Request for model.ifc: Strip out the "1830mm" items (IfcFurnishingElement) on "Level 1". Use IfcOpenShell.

First a look at what the model holds.

```python
import ifcopenshell
import ifcopenshell.util.element

model = ifcopenshell.open("model.ifc")
print(model.schema)
storey = next(s for s in model.by_type("IfcBuildingStorey") if s.Name == "Level 1")
furniture = [e for e in ifcopenshell.util.element.get_decomposition(storey) if e.is_a("IfcFurnishingElement")]
seen = {}
for e in furniture:
    element_type = ifcopenshell.util.element.get_type(e)
    name = element_type.Name if element_type not in (None, e) else None
    seen[name] = seen.get(name, 0) + 1
for name, count in sorted(seen.items(), key=str):
    print(count, "x", name)
```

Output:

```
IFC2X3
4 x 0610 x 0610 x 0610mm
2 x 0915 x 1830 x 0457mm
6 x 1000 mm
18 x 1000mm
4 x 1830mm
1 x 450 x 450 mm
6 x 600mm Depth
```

```python
import ifcopenshell
import ifcopenshell.api.root
import ifcopenshell.util.element

model = ifcopenshell.open("model.ifc")

storey = next(s for s in model.by_type("IfcBuildingStorey") if s.Name == "Level 1")
furniture = [e for e in ifcopenshell.util.element.get_decomposition(storey) if e.is_a("IfcFurnishingElement")]
targets = [e for e in furniture if (t := ifcopenshell.util.element.get_type(e)) not in (None, e) and t.Name == "1830mm"]

for e in targets:
    ifcopenshell.api.root.remove_product(model, product=e)
print(len(targets), "removed")

model.write("model_rev.ifc")
```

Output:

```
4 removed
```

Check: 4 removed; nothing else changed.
